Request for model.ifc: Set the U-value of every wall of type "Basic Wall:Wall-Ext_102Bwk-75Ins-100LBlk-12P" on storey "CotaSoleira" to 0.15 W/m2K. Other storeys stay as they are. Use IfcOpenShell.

First a look at what the model holds.

```python
import ifcopenshell
import ifcopenshell.util.element

model = ifcopenshell.open("model.ifc")
print(model.schema)
storey = next(s for s in model.by_type("IfcBuildingStorey") if s.Name == "CotaSoleira")
walls = [e for e in ifcopenshell.util.element.get_decomposition(storey) if e.is_a("IfcWall")]
seen = {}
for e in walls:
    element_type = ifcopenshell.util.element.get_type(e)
    key = (element_type.Name if element_type != e and element_type else None, ifcopenshell.util.element.get_pset(e, "Pset_WallCommon", "ThermalTransmittance"))
    seen[key] = seen.get(key, 0) + 1
for (name, value), count in sorted(seen.items(), key=str):
    print(count, "x", name, "|", value)
```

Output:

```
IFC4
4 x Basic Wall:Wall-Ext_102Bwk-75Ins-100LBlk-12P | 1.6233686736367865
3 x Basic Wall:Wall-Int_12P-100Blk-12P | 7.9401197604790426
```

```python
import ifcopenshell
import ifcopenshell.api.pset
import ifcopenshell.util.element

model = ifcopenshell.open("model.ifc")

storey = next(s for s in model.by_type("IfcBuildingStorey") if s.Name == "CotaSoleira")
walls = [e for e in ifcopenshell.util.element.get_decomposition(storey) if e.is_a("IfcWall")]

count = 0
for e in walls:
    element_type = ifcopenshell.util.element.get_type(e)
    if element_type in (None, e) or element_type.Name != "Basic Wall:Wall-Ext_102Bwk-75Ins-100LBlk-12P":
        continue
    # add_pset returns the element's existing set when there is one.
    pset = ifcopenshell.api.pset.add_pset(model, product=e, name="Pset_WallCommon")
    ifcopenshell.api.pset.edit_pset(model, pset=pset, properties={"ThermalTransmittance": 0.15})
    count += 1

print(count, "walls updated")

model.write("model_edited.ifc")
```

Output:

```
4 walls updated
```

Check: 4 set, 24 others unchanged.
